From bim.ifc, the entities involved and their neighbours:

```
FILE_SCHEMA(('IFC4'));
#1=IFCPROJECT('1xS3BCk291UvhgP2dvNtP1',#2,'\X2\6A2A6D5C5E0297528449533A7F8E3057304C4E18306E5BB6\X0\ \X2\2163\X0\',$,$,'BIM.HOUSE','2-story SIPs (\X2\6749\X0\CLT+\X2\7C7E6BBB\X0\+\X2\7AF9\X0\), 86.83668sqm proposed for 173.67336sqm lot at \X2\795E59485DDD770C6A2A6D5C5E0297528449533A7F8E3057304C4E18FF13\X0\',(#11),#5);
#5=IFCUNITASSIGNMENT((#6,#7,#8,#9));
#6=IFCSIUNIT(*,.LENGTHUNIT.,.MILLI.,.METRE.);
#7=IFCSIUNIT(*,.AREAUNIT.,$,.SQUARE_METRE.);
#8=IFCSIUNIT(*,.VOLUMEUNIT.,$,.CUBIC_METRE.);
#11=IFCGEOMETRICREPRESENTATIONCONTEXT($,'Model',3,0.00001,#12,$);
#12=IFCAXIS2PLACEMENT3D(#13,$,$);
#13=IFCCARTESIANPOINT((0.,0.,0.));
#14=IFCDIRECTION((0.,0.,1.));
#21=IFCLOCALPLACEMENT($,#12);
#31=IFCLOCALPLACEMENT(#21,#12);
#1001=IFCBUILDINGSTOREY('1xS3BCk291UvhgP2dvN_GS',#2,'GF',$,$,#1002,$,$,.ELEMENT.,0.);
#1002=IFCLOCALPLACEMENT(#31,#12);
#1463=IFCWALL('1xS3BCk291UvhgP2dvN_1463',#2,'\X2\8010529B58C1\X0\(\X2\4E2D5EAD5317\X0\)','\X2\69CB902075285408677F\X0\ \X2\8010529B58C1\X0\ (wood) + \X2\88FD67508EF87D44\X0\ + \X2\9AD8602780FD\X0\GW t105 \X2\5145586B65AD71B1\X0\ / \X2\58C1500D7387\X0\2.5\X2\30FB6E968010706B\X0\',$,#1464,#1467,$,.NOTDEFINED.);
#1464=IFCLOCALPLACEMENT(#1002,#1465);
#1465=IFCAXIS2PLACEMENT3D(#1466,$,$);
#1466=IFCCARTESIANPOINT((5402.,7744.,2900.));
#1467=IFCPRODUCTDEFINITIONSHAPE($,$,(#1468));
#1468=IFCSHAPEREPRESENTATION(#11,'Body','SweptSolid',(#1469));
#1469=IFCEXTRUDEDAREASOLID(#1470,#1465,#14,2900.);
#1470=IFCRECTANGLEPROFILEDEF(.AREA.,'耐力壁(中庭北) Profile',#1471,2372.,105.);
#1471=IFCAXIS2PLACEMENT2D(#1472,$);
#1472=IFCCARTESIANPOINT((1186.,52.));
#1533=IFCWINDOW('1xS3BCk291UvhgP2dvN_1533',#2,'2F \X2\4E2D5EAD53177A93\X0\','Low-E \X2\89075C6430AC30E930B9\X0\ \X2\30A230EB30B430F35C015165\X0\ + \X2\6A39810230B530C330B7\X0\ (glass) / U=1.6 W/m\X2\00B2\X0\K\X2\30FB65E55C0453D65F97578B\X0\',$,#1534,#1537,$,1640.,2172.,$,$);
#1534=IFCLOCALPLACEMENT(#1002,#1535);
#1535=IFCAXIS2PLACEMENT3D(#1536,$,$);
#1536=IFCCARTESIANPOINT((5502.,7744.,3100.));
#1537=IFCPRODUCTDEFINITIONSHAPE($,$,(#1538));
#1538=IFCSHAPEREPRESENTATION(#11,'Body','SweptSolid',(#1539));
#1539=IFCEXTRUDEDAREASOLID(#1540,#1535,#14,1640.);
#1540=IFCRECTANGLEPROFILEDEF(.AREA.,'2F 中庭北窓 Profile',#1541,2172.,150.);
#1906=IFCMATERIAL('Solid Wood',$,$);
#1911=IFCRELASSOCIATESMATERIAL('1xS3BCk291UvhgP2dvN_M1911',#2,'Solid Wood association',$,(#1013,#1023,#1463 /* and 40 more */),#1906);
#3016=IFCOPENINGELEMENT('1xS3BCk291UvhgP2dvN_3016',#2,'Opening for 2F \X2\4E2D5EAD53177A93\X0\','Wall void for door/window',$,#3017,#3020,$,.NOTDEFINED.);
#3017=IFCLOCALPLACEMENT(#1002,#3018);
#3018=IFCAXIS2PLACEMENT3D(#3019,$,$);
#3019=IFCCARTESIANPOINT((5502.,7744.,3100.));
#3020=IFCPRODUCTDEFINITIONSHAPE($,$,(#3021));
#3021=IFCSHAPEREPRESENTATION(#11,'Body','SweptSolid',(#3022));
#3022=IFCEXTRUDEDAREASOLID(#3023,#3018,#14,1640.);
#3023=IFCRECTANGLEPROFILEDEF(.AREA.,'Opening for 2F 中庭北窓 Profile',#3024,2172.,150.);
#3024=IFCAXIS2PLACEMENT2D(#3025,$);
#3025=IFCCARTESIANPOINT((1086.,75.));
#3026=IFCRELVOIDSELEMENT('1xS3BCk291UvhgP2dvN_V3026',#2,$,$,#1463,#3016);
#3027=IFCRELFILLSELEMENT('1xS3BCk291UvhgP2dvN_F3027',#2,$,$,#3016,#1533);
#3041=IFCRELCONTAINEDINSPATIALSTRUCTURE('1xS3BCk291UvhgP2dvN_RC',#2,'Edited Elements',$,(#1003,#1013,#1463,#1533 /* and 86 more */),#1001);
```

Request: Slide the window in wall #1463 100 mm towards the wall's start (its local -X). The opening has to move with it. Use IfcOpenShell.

```python
import ifcopenshell
import ifcopenshell.api.geometry
import ifcopenshell.util.placement

model = ifcopenshell.open("bim.ifc")

window = model.by_guid("1xS3BCk291UvhgP2dvN_1533")
opening = window.FillsVoids[0].RelatingOpeningElement
wall = opening.VoidsElements[0].RelatingBuildingElement

wall_matrix = ifcopenshell.util.placement.get_local_placement(wall.ObjectPlacement)
shift = wall_matrix[:3, 0] * -100.0
before = ifcopenshell.util.placement.get_local_placement(window.ObjectPlacement)[:3, 3].copy()

# The window is not placed relative to its opening, so move both.
for product in (opening, window):
    matrix = ifcopenshell.util.placement.get_local_placement(product.ObjectPlacement)
    matrix[:3, 3] += shift
    ifcopenshell.api.geometry.edit_object_placement(model, product=product, matrix=matrix, is_si=False)

after = ifcopenshell.util.placement.get_local_placement(window.ObjectPlacement)[:3, 3]
print("window moved by", (after - before).round(3) + 0.0)

model.write("bim_updated.ifc")
```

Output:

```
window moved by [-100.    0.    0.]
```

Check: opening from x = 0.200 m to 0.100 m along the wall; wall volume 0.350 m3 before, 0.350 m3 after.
